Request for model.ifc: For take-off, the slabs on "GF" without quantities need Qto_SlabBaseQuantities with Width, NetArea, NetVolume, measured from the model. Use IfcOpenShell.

First a look at what the model holds.

```python
import ifcopenshell
import ifcopenshell.util.element
import ifcopenshell.util.unit

model = ifcopenshell.open("model.ifc")
print(model.schema)
for unit_type in ("LENGTHUNIT", "AREAUNIT", "VOLUMEUNIT"):
    print(unit_type, ifcopenshell.util.unit.calculate_unit_scale(model, unit_type))
storey = next(s for s in model.by_type("IfcBuildingStorey") if s.Name == "GF")
slabs = [e for e in ifcopenshell.util.element.get_decomposition(storey) if e.is_a("IfcSlab")]
for e in sorted(slabs, key=lambda e: e.id()):
    print(e.id(), e.is_a(), e.Name, list(ifcopenshell.util.element.get_psets(e, qtos_only=True)), sep=" | ")
```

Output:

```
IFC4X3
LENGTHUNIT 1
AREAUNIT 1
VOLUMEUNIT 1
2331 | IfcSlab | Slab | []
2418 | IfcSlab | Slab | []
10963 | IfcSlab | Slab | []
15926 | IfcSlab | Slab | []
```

```python
import ifcopenshell
import ifcopenshell.api.pset
import ifcopenshell.geom
import ifcopenshell.util.element
import ifcopenshell.util.shape
import ifcopenshell.util.unit

model = ifcopenshell.open("model.ifc")
unit_scale = ifcopenshell.util.unit.calculate_unit_scale(model)
area_scale = ifcopenshell.util.unit.calculate_unit_scale(model, "AREAUNIT")
volume_scale = ifcopenshell.util.unit.calculate_unit_scale(model, "VOLUMEUNIT")
settings = ifcopenshell.geom.settings()

storey = next(s for s in model.by_type("IfcBuildingStorey") if s.Name == "GF")
slabs = [e for e in ifcopenshell.util.element.get_decomposition(storey) if e.is_a("IfcSlab")]

for e in sorted(slabs, key=lambda e: e.id()):
    if ifcopenshell.util.element.get_psets(e, qtos_only=True, should_inherit=False):
        continue
    # Geometry comes back in metres, in the element's own axes.
    shape = ifcopenshell.geom.create_shape(settings, e)
    values = {
        "Width": ifcopenshell.util.shape.get_z(shape.geometry) / unit_scale,
        "NetArea": ifcopenshell.util.shape.get_footprint_area(shape.geometry) / area_scale,
        "NetVolume": ifcopenshell.util.shape.get_volume(shape.geometry) / volume_scale,
    }
    qto = ifcopenshell.api.pset.add_qto(model, product=e, name="Qto_SlabBaseQuantities")
    ifcopenshell.api.pset.edit_qto(model, qto=qto, properties=values)
    print(e.id(), {k: round(v, 3) for k, v in values.items()})

model.write("model_updated.ifc")
```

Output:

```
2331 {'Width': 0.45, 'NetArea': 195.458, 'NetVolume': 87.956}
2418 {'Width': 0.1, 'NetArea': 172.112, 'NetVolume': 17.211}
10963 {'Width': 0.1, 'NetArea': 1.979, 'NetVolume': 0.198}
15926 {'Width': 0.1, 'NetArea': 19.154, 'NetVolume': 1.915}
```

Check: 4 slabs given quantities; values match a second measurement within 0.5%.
